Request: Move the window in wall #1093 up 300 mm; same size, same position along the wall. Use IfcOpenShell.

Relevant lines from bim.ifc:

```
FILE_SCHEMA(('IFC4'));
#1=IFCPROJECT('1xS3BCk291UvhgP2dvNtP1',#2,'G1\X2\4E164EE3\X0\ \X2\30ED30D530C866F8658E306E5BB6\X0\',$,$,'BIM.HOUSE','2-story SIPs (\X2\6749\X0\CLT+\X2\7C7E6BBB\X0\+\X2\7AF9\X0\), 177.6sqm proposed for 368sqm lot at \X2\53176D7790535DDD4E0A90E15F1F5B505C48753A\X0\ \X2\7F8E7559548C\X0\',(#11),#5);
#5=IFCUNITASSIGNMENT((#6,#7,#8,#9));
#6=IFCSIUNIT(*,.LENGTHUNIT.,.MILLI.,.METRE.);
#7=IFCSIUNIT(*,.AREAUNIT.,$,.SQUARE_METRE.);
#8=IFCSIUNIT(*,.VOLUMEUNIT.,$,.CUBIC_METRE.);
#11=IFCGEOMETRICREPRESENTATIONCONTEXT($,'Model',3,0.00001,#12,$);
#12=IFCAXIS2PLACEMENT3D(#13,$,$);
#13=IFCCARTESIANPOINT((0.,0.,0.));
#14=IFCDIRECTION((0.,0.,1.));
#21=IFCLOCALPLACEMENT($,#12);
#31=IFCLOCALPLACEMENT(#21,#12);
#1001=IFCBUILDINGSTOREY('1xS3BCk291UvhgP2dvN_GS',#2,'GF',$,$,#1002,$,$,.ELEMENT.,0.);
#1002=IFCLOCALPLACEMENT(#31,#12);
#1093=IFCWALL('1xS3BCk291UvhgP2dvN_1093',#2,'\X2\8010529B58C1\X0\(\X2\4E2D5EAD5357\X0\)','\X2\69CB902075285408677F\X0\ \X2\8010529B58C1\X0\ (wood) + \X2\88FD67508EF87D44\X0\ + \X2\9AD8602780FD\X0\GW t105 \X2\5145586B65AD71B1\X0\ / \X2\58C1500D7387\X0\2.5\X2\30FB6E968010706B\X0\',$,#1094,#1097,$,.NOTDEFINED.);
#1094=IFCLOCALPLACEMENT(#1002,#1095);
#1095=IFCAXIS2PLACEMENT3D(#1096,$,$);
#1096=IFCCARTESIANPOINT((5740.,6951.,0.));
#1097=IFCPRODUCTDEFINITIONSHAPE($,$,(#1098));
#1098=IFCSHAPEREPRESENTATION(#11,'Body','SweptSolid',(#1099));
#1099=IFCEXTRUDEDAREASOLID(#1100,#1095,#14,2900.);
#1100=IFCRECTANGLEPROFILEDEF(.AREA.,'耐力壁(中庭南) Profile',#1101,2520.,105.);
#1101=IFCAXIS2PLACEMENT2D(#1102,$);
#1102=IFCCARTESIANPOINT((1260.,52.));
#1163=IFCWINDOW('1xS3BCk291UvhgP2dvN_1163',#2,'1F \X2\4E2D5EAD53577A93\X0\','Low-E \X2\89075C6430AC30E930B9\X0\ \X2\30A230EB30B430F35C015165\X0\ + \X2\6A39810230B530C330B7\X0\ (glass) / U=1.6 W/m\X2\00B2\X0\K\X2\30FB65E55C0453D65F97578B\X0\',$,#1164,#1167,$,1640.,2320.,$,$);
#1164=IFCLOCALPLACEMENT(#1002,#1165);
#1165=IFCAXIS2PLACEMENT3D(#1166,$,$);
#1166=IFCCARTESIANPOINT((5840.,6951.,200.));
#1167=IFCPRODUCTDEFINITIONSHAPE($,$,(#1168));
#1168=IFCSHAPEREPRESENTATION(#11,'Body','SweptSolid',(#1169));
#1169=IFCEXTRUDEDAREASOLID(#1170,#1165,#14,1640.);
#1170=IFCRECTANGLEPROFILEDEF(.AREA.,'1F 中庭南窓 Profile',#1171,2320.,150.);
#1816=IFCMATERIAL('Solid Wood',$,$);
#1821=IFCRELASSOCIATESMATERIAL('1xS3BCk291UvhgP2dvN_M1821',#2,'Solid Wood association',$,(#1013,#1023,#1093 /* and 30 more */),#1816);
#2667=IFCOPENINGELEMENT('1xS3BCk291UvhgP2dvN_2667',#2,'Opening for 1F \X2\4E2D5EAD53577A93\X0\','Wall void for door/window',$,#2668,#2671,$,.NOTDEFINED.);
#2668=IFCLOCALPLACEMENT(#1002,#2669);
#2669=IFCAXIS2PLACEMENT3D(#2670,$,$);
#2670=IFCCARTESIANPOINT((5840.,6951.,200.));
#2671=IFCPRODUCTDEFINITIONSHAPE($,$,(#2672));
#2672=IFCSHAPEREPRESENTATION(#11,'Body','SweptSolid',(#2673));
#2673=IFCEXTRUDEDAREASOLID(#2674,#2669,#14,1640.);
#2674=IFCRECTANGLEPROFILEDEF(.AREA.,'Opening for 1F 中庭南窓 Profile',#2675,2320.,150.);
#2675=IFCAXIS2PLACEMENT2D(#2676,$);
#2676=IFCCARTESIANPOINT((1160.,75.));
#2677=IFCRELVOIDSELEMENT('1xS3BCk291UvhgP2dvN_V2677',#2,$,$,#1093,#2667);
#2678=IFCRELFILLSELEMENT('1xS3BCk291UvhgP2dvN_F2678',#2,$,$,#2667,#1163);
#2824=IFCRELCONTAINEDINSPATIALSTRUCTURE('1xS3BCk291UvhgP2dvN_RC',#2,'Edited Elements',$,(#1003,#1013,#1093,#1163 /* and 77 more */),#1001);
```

```python
import numpy as np
import ifcopenshell
import ifcopenshell.api.geometry
import ifcopenshell.util.placement
import ifcopenshell.util.unit

model = ifcopenshell.open("bim.ifc")
unit_scale = ifcopenshell.util.unit.calculate_unit_scale(model)

window = model.by_guid("1xS3BCk291UvhgP2dvN_1163")
opening = window.FillsVoids[0].RelatingOpeningElement
dz = 0.3 / unit_scale

shift = np.array([0.0, 0.0, dz])
# The window is not placed relative to its opening, so move both.
for product in (opening, window):
    matrix = ifcopenshell.util.placement.get_local_placement(product.ObjectPlacement)
    matrix[:3, 3] += shift
    ifcopenshell.api.geometry.edit_object_placement(model, product=product, matrix=matrix, is_si=False)

print(f"moved by {dz * unit_scale:+.3f} m")

model.write("bim-out.ifc")
```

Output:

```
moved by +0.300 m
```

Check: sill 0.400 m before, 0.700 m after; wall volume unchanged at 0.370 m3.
